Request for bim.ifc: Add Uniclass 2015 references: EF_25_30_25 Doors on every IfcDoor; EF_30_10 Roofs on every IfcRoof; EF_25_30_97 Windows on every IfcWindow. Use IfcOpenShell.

First a look at what the model holds.

```python
import ifcopenshell

model = ifcopenshell.open("bim.ifc")
print(model.schema)
print("classifications:", [c.Name for c in model.by_type("IfcClassification")])
for ifc_class in ("IfcDoor", "IfcRoof", "IfcStair", "IfcWall", "IfcWindow"):
    print(ifc_class, len(model.by_type(ifc_class)))
```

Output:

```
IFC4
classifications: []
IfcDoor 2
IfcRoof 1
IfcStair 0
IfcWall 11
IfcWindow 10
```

```python
import ifcopenshell
import ifcopenshell.api.classification

model = ifcopenshell.open("bim.ifc")

system = ifcopenshell.api.classification.add_classification(model, classification="Uniclass 2015")

codes = {
    "IfcDoor": ("EF_25_30_25", "Doors"),
    "IfcRoof": ("EF_30_10", "Roofs"),
    "IfcWindow": ("EF_25_30_97", "Windows"),
}
for ifc_class, (code, name) in codes.items():
    products = model.by_type(ifc_class)
    ifcopenshell.api.classification.add_reference(
        model, products=products, classification=system, identification=code, name=name
    )
    print(code, len(products))

model.write("bim-out.ifc")
```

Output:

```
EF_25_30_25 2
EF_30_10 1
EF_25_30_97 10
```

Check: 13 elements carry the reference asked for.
